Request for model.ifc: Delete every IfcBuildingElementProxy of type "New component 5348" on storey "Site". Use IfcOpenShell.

First a look at what the model holds.

```python
import ifcopenshell
import ifcopenshell.util.element

model = ifcopenshell.open("model.ifc")
print(model.schema)
storey = next(s for s in model.by_type("IfcBuildingStorey") if s.Name == "Site")
proxies = [e for e in ifcopenshell.util.element.get_decomposition(storey) if e.is_a("IfcBuildingElementProxy")]
seen = {}
for e in proxies:
    element_type = ifcopenshell.util.element.get_type(e)
    name = element_type.Name if element_type not in (None, e) else None
    seen[name] = seen.get(name, 0) + 1
for name, count in sorted(seen.items(), key=str):
    print(count, "x", name)
```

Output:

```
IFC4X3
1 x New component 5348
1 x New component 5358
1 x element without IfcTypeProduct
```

```python
import ifcopenshell
import ifcopenshell.api.root
import ifcopenshell.util.element

model = ifcopenshell.open("model.ifc")

storey = next(s for s in model.by_type("IfcBuildingStorey") if s.Name == "Site")
proxies = [e for e in ifcopenshell.util.element.get_decomposition(storey) if e.is_a("IfcBuildingElementProxy")]
targets = [e for e in proxies if (t := ifcopenshell.util.element.get_type(e)) not in (None, e) and t.Name == "New component 5348"]

for e in targets:
    ifcopenshell.api.root.remove_product(model, product=e)
print(len(targets), "removed")

model.write("model_updated.ifc")
```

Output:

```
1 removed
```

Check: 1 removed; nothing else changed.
